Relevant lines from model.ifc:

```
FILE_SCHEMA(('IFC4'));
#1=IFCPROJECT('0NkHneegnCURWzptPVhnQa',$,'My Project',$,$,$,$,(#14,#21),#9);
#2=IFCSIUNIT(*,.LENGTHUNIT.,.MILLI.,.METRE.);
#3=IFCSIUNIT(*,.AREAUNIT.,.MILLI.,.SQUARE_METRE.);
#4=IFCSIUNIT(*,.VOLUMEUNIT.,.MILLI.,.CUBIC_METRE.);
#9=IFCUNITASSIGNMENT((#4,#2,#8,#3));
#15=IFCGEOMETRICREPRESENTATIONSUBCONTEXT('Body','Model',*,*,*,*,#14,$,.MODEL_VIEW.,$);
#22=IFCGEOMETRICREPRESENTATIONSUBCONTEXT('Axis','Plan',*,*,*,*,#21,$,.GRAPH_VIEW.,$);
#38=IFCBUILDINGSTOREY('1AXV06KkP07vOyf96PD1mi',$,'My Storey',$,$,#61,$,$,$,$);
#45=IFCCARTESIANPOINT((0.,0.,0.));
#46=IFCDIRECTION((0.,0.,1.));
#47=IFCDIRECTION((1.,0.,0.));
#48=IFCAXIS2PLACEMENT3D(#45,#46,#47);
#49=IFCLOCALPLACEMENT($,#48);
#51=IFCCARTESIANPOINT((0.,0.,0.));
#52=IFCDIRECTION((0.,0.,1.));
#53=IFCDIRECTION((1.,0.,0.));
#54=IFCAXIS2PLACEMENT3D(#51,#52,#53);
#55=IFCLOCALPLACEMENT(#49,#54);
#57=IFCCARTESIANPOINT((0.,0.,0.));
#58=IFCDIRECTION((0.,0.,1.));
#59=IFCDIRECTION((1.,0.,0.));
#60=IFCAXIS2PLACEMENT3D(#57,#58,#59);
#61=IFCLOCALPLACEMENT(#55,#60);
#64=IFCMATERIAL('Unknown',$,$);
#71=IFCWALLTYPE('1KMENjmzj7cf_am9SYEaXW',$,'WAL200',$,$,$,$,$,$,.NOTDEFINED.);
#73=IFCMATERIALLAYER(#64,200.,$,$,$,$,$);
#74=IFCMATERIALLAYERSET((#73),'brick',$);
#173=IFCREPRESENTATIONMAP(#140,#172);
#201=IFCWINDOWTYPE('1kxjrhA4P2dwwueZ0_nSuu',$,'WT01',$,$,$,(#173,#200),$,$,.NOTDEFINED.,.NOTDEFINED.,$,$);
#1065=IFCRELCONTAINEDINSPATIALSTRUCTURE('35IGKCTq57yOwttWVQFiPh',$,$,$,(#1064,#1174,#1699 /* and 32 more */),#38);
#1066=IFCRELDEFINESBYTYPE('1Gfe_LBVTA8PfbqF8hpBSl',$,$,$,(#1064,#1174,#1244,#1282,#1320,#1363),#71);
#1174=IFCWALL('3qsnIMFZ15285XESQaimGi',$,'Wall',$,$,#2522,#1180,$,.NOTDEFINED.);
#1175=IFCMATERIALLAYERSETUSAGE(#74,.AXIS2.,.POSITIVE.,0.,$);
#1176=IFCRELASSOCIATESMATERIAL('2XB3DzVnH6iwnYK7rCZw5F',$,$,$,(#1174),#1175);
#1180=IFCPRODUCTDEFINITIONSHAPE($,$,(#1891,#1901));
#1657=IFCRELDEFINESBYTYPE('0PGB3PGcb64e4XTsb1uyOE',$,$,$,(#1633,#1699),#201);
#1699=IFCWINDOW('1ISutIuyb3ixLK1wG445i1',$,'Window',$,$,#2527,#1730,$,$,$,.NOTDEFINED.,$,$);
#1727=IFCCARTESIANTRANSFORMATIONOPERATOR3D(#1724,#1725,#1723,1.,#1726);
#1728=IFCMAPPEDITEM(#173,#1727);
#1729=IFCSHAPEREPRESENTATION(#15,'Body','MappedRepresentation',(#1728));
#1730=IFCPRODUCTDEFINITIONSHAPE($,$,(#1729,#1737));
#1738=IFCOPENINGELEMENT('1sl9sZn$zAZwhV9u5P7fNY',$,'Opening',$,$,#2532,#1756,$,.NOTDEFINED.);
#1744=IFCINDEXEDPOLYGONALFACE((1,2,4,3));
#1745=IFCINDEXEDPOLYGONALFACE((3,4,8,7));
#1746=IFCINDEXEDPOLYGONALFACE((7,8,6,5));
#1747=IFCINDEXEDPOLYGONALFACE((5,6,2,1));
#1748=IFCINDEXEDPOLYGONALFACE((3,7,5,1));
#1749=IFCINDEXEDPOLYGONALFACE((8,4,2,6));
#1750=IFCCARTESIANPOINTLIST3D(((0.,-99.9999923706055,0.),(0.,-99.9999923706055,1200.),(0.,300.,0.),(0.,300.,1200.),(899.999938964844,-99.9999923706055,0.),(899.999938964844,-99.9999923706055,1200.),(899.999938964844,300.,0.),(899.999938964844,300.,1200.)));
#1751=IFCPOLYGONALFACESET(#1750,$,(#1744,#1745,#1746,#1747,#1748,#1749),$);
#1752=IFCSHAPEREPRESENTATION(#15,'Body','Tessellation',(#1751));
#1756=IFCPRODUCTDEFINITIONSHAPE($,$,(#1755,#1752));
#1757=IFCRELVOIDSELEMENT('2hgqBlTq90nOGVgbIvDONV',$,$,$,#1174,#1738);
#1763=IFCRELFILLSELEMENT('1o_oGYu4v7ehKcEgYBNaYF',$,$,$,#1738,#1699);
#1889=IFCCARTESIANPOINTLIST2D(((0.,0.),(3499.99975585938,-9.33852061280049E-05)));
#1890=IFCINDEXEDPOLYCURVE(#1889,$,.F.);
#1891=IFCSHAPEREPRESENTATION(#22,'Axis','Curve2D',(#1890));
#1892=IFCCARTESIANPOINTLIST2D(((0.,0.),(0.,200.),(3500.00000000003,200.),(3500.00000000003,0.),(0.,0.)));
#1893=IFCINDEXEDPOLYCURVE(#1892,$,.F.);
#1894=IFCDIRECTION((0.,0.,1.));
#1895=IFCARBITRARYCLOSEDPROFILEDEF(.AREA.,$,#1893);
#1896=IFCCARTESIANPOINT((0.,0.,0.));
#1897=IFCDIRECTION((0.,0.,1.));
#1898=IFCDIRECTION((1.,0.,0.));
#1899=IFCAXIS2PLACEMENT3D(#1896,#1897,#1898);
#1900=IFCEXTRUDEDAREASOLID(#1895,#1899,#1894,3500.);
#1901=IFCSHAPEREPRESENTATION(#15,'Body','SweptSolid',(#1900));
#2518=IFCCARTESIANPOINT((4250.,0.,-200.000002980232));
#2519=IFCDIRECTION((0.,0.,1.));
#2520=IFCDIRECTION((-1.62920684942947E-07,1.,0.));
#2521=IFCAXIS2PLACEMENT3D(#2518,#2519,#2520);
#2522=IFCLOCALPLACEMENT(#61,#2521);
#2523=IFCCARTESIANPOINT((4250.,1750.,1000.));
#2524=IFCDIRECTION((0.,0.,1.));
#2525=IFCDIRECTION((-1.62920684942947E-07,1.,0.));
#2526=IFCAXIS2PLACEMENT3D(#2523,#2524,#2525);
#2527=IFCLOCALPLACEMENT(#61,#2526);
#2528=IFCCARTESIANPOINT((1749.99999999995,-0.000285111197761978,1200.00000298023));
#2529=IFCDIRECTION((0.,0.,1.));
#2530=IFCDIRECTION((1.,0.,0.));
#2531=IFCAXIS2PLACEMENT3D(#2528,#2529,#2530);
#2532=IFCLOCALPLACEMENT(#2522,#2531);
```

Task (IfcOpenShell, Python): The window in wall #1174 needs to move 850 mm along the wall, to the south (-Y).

```python
import ifcopenshell
import ifcopenshell.api.geometry
import ifcopenshell.util.placement
import ifcopenshell.util.unit

model = ifcopenshell.open("model.ifc")
unit_scale = ifcopenshell.util.unit.calculate_unit_scale(model)

window = model.by_guid("1ISutIuyb3ixLK1wG445i1")
opening = window.FillsVoids[0].RelatingOpeningElement
wall = opening.VoidsElements[0].RelatingBuildingElement

wall_matrix = ifcopenshell.util.placement.get_local_placement(wall.ObjectPlacement)
shift = wall_matrix[:3, 0] * -0.85 / unit_scale
before = ifcopenshell.util.placement.get_local_placement(window.ObjectPlacement)[:3, 3].copy()

# The window is not placed relative to its opening, so move both.
for product in (opening, window):
    matrix = ifcopenshell.util.placement.get_local_placement(product.ObjectPlacement)
    matrix[:3, 3] += shift
    ifcopenshell.api.geometry.edit_object_placement(model, product=product, matrix=matrix, is_si=False)

after = ifcopenshell.util.placement.get_local_placement(window.ObjectPlacement)[:3, 3]
print("window moved by", (after - before).round(3) + 0.0)

model.write("model_v2.ifc")
```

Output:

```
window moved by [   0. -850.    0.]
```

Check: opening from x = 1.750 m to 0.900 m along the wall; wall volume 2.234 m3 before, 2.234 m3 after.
